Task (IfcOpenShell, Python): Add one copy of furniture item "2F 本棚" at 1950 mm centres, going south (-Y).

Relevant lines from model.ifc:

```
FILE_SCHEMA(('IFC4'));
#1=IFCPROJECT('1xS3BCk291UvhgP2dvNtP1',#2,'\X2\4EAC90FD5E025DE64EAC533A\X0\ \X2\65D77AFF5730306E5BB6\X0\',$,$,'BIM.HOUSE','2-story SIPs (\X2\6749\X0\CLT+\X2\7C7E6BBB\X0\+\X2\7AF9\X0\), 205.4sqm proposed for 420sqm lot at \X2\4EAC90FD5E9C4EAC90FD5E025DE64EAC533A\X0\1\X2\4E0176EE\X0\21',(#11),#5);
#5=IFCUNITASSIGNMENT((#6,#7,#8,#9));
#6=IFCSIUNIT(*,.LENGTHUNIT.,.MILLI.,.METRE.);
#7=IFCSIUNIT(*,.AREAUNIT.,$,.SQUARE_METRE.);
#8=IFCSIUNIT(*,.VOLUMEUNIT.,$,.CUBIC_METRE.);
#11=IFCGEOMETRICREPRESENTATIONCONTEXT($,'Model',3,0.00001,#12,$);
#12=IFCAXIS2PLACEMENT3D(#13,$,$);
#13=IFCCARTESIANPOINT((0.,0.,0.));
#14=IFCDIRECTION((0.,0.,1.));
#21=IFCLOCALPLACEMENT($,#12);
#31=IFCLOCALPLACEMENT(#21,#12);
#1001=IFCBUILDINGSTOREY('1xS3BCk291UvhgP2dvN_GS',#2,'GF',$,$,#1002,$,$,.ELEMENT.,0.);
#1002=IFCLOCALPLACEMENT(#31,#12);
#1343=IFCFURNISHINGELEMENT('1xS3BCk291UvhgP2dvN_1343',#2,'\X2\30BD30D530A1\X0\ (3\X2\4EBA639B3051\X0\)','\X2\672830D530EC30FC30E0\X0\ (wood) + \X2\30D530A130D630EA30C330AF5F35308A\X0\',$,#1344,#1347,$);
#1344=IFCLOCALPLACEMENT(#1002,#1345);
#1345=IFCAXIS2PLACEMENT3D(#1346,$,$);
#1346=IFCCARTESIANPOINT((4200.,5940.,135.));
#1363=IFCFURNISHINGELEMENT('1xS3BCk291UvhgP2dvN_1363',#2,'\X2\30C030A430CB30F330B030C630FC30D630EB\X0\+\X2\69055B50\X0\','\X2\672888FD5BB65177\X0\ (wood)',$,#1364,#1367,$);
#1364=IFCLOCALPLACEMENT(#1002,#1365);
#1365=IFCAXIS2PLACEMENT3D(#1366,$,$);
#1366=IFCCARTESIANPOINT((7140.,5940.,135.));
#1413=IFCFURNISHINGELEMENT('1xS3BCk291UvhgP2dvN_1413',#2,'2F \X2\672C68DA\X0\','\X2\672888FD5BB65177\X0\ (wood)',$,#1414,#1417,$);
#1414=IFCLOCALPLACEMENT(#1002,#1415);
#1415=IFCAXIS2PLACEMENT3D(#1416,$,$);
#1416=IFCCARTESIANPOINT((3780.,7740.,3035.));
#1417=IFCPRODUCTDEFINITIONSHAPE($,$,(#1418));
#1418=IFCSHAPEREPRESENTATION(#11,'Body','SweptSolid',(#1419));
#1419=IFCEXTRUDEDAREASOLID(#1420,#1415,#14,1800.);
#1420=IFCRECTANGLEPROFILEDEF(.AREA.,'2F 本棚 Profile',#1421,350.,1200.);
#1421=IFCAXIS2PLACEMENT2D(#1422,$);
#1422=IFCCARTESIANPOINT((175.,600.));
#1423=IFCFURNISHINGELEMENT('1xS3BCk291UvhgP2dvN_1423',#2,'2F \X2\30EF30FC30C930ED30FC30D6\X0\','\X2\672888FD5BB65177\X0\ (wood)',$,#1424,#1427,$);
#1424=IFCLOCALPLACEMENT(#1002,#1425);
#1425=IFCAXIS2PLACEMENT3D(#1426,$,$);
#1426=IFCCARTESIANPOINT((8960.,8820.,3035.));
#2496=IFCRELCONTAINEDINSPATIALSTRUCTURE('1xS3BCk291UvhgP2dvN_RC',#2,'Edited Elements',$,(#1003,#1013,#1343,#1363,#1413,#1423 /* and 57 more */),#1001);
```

```python
import numpy as np
import ifcopenshell
import ifcopenshell.api.geometry
import ifcopenshell.api.root
import ifcopenshell.util.element
import ifcopenshell.util.placement
import ifcopenshell.util.unit

model = ifcopenshell.open("model.ifc")
unit_scale = ifcopenshell.util.unit.calculate_unit_scale(model)


def reuse_history(source, copy):
    """copy_class also copies each property set's owner history, people and application; keep the originals."""
    for rel in copy.IsDefinedBy:
        if rel.is_a("IfcRelDefinesByProperties") and (history := rel.RelatingPropertyDefinition.OwnerHistory):
            rel.RelatingPropertyDefinition.OwnerHistory = source.OwnerHistory
            ifcopenshell.util.element.remove_deep2(model, history)


source = model.by_guid("1xS3BCk291UvhgP2dvN_1413")
base = ifcopenshell.util.placement.get_local_placement(source.ObjectPlacement)
step = np.array([0.0, -1.0, 0.0]) * 1.95 / unit_scale

for i in range(1, 2):
    copy = ifcopenshell.api.root.copy_class(model, product=source)
    copy.Representation = ifcopenshell.util.element.copy_deep(
        model, source.Representation, exclude=["IfcGeometricRepresentationContext", "IfcRepresentationMap"]
    )
    reuse_history(source, copy)
    matrix = base.copy()
    matrix[:3, 3] += i * step
    print("added at", matrix[:3, 3].round(3) + 0.0)
    ifcopenshell.api.geometry.edit_object_placement(model, product=copy, matrix=matrix, is_si=False)

model.write("model_rev.ifc")
```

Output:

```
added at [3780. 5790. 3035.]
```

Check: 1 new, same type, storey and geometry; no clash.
